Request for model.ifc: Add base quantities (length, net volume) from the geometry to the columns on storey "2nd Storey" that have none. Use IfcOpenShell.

First a look at what the model holds.

```python
import ifcopenshell
import ifcopenshell.util.element
import ifcopenshell.util.unit

model = ifcopenshell.open("model.ifc")
print(model.schema)
for unit_type in ("LENGTHUNIT", "AREAUNIT", "VOLUMEUNIT"):
    print(unit_type, ifcopenshell.util.unit.calculate_unit_scale(model, unit_type))
storey = next(s for s in model.by_type("IfcBuildingStorey") if s.Name == "2nd Storey")
columns = [e for e in ifcopenshell.util.element.get_decomposition(storey) if e.is_a("IfcColumn")]
for e in sorted(columns, key=lambda e: e.id()):
    print(e.id(), e.is_a(), e.Name, list(ifcopenshell.util.element.get_psets(e, qtos_only=True)), sep=" | ")
```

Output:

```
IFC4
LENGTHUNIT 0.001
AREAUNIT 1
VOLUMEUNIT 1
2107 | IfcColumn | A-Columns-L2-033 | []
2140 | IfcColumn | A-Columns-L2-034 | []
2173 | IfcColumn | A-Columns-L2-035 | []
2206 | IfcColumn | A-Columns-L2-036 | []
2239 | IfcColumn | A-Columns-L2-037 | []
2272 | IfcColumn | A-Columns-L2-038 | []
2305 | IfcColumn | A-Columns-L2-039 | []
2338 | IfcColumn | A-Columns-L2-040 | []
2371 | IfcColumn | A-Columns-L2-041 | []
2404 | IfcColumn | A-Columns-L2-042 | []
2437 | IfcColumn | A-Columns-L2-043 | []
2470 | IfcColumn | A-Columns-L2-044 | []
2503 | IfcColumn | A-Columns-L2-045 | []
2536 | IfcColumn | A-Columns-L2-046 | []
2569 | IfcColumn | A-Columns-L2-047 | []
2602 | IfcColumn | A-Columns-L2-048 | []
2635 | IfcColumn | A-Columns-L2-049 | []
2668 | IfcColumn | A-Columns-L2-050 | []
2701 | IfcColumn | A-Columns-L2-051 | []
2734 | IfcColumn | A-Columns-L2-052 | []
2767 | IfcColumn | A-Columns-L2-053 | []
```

```python
import ifcopenshell
import ifcopenshell.api.pset
import ifcopenshell.geom
import ifcopenshell.util.element
import ifcopenshell.util.shape
import ifcopenshell.util.unit

model = ifcopenshell.open("model.ifc")
unit_scale = ifcopenshell.util.unit.calculate_unit_scale(model)
volume_scale = ifcopenshell.util.unit.calculate_unit_scale(model, "VOLUMEUNIT")
settings = ifcopenshell.geom.settings()

storey = next(s for s in model.by_type("IfcBuildingStorey") if s.Name == "2nd Storey")
columns = [e for e in ifcopenshell.util.element.get_decomposition(storey) if e.is_a("IfcColumn")]

for e in sorted(columns, key=lambda e: e.id()):
    if ifcopenshell.util.element.get_psets(e, qtos_only=True, should_inherit=False):
        continue
    # Geometry comes back in metres, in the element's own axes.
    shape = ifcopenshell.geom.create_shape(settings, e)
    values = {
        "Length": ifcopenshell.util.shape.get_z(shape.geometry) / unit_scale,
        "NetVolume": ifcopenshell.util.shape.get_volume(shape.geometry) / volume_scale,
    }
    qto = ifcopenshell.api.pset.add_qto(model, product=e, name="Qto_ColumnBaseQuantities")
    ifcopenshell.api.pset.edit_qto(model, qto=qto, properties=values)
    print(e.id(), {k: round(v, 3) for k, v in values.items()})

model.write("model-out.ifc")
```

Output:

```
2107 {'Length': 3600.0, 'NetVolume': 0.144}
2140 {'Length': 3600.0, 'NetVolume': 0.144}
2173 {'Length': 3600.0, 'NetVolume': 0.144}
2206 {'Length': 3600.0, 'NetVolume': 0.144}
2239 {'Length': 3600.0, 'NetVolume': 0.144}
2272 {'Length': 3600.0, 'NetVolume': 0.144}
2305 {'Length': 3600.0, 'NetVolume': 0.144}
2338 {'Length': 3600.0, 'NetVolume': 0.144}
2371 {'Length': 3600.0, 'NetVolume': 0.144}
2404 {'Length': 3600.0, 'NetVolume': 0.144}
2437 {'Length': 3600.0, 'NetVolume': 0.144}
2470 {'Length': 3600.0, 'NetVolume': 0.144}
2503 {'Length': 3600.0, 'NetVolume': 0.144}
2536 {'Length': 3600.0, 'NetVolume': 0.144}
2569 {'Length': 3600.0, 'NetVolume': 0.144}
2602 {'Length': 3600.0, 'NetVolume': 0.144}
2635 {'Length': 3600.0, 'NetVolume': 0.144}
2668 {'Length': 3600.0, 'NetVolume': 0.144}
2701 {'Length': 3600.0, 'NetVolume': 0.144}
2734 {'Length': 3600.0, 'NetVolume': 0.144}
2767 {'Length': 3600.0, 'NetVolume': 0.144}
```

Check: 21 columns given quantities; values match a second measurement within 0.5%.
